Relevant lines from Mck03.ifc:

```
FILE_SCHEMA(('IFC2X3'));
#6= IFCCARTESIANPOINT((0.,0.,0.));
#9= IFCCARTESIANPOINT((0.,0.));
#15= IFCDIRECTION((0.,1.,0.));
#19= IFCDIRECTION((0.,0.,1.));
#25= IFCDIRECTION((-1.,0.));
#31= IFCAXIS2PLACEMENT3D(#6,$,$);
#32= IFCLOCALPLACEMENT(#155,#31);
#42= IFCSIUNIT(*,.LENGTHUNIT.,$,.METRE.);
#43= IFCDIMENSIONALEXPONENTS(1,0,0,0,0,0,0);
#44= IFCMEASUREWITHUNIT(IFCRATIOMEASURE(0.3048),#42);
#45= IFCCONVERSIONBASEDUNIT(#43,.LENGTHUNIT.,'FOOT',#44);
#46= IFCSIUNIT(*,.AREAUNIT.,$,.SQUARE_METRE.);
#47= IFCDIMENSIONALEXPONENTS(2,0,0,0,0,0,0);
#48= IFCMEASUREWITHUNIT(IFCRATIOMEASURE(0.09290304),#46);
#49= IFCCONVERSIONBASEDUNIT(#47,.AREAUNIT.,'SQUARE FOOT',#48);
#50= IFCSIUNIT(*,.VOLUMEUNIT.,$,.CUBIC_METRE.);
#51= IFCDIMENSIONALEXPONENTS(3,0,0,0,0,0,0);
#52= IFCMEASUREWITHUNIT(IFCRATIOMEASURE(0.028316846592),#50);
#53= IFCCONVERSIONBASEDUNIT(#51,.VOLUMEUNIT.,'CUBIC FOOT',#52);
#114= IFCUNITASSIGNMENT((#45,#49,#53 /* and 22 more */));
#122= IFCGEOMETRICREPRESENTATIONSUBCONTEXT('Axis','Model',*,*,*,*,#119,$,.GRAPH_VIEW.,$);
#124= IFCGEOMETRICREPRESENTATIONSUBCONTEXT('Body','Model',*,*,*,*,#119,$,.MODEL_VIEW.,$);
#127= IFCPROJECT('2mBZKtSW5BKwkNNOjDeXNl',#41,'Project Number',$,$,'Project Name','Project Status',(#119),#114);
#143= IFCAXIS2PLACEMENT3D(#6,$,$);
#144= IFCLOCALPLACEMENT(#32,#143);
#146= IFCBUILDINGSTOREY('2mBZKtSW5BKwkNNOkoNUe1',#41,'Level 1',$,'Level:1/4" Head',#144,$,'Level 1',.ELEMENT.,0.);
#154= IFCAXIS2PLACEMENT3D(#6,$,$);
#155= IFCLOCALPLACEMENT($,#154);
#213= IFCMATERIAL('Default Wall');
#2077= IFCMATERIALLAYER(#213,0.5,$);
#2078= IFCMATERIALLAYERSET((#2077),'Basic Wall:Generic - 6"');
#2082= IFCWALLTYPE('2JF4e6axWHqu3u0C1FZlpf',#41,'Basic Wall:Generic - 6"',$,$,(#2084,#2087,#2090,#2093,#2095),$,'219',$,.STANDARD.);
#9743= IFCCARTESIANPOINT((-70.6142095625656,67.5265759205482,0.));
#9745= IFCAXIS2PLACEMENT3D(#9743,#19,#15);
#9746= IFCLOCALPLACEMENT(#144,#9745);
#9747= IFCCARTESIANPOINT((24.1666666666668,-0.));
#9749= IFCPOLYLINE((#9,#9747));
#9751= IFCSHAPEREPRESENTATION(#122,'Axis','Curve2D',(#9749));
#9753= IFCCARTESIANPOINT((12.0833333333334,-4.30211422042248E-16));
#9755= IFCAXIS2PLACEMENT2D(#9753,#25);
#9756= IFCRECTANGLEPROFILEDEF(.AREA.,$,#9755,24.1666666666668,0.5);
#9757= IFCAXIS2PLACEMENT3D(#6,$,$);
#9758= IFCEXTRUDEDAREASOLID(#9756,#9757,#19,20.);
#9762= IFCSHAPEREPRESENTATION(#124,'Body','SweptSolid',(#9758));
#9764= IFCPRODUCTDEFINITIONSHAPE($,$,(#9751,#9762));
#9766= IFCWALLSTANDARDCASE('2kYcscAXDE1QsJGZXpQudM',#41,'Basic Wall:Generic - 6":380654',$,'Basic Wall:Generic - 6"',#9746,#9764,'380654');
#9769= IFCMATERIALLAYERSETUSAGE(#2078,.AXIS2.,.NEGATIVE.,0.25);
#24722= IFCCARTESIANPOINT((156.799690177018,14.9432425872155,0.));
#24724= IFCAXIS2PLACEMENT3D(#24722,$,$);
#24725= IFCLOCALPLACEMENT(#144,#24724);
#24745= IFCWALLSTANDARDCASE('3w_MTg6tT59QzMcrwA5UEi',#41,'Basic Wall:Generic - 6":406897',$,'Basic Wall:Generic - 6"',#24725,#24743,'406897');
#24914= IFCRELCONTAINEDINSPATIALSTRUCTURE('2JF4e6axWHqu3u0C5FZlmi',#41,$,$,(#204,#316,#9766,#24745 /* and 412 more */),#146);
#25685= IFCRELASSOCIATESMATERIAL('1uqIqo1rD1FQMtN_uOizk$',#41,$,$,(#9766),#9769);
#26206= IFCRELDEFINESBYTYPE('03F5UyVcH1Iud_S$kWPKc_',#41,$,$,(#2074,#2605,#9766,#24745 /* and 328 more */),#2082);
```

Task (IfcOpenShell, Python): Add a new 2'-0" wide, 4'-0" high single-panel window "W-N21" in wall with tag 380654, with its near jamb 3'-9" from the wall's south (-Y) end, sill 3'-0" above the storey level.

```python
import numpy as np
import ifcopenshell
import ifcopenshell.api.feature
import ifcopenshell.api.geometry
import ifcopenshell.api.root
import ifcopenshell.api.spatial
import ifcopenshell.api.type
import ifcopenshell.geom
import ifcopenshell.util.element
import ifcopenshell.util.placement
import ifcopenshell.util.representation
import ifcopenshell.util.shape
import ifcopenshell.util.unit

model = ifcopenshell.open("Mck03.ifc")
unit_scale = ifcopenshell.util.unit.calculate_unit_scale(model)
settings = ifcopenshell.geom.settings()


def volume(element):
    """Net volume in cubic metres, openings subtracted."""
    shape = ifcopenshell.geom.create_shape(settings, element)
    return ifcopenshell.util.shape.get_volume(shape.geometry)


wall = model.by_guid("2kYcscAXDE1QsJGZXpQudM")
storey = ifcopenshell.util.element.get_container(wall, ifc_class="IfcBuildingStorey")
context = ifcopenshell.util.representation.get_context(model, "Model", "Body", "MODEL_VIEW")
before = volume(wall)

width, height, from_end, sill = 0.6096, 1.2192, 1.143, 0.9144  # metres

# The wall runs along its own X axis, and the end named is its -X end.
wall_shape = ifcopenshell.geom.create_shape(settings, wall)
x, y, z = ifcopenshell.util.shape.get_vertices(wall_shape.geometry).T
start = x.min() + from_end
face, thickness = float(y.min()), float(y.max() - y.min())
wall_matrix = ifcopenshell.util.placement.get_local_placement(wall.ObjectPlacement)
level = ifcopenshell.util.placement.get_local_placement(storey.ObjectPlacement)[2, 3]


def in_wall(x, y):
    """Placement at x, y metres in the wall's axes, at sill height."""
    matrix = wall_matrix.copy()
    matrix[:, 3] = wall_matrix @ np.array([x / unit_scale, y / unit_scale, 0.0, 1.0])
    matrix[2, 3] = level + sill / unit_scale
    return matrix


# Opening: a box that overshoots both wall faces by 50 mm.
opening = ifcopenshell.api.root.create_entity(model, ifc_class="IfcOpeningElement")
box = ifcopenshell.api.geometry.add_wall_representation(
    model, context=context, length=width, height=height, thickness=thickness + 0.1
)
ifcopenshell.api.geometry.assign_representation(model, product=opening, representation=box)
ifcopenshell.api.geometry.edit_object_placement(model, product=opening, matrix=in_wall(start, face - 0.05), is_si=False)
ifcopenshell.api.feature.add_feature(model, feature=opening, element=wall)

window = ifcopenshell.api.root.create_entity(model, ifc_class="IfcWindow", name="W-N21")
window.OverallWidth, window.OverallHeight = width / unit_scale, height / unit_scale
body = ifcopenshell.api.geometry.add_window_representation(
    model,
    context=context,
    overall_width=window.OverallWidth,
    overall_height=window.OverallHeight,
    partition_type="SINGLE_PANEL",
)
ifcopenshell.api.geometry.assign_representation(model, product=window, representation=body)
ifcopenshell.api.spatial.assign_container(model, products=[window], relating_structure=storey)
fills = ifcopenshell.api.feature.add_filling(model, opening=opening, element=window)
fills.OwnerHistory = window.OwnerHistory  # required in IFC2X3

# IFC2X3 keeps the operation on the window style.
style = ifcopenshell.api.root.create_entity(model, ifc_class="IfcWindowStyle", name="W-N21")
style.OperationType, style.ConstructionType = "SINGLE_PANEL", "NOTDEFINED"
style.ParameterTakesPrecedence = style.Sizeable = False
ifcopenshell.api.type.assign_type(model, related_objects=[window], relating_type=style)

# Centre the window in the wall's thickness.
ifcopenshell.api.geometry.edit_object_placement(model, product=window, matrix=in_wall(start, face), is_si=False)
window_shape = ifcopenshell.geom.create_shape(settings, window)
depth = ifcopenshell.util.shape.get_vertices(window_shape.geometry)[:, 1]
offset = face + thickness / 2 - (depth.min() + depth.max()) / 2
ifcopenshell.api.geometry.edit_object_placement(model, product=window, matrix=in_wall(start, offset), is_si=False)

after = volume(wall)

print(f"wall volume {before:.3f} -> {after:.3f} m3")

model.write("Mck03-out.ifc")
```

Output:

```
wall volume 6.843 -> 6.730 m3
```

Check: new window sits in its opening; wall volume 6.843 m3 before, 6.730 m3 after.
